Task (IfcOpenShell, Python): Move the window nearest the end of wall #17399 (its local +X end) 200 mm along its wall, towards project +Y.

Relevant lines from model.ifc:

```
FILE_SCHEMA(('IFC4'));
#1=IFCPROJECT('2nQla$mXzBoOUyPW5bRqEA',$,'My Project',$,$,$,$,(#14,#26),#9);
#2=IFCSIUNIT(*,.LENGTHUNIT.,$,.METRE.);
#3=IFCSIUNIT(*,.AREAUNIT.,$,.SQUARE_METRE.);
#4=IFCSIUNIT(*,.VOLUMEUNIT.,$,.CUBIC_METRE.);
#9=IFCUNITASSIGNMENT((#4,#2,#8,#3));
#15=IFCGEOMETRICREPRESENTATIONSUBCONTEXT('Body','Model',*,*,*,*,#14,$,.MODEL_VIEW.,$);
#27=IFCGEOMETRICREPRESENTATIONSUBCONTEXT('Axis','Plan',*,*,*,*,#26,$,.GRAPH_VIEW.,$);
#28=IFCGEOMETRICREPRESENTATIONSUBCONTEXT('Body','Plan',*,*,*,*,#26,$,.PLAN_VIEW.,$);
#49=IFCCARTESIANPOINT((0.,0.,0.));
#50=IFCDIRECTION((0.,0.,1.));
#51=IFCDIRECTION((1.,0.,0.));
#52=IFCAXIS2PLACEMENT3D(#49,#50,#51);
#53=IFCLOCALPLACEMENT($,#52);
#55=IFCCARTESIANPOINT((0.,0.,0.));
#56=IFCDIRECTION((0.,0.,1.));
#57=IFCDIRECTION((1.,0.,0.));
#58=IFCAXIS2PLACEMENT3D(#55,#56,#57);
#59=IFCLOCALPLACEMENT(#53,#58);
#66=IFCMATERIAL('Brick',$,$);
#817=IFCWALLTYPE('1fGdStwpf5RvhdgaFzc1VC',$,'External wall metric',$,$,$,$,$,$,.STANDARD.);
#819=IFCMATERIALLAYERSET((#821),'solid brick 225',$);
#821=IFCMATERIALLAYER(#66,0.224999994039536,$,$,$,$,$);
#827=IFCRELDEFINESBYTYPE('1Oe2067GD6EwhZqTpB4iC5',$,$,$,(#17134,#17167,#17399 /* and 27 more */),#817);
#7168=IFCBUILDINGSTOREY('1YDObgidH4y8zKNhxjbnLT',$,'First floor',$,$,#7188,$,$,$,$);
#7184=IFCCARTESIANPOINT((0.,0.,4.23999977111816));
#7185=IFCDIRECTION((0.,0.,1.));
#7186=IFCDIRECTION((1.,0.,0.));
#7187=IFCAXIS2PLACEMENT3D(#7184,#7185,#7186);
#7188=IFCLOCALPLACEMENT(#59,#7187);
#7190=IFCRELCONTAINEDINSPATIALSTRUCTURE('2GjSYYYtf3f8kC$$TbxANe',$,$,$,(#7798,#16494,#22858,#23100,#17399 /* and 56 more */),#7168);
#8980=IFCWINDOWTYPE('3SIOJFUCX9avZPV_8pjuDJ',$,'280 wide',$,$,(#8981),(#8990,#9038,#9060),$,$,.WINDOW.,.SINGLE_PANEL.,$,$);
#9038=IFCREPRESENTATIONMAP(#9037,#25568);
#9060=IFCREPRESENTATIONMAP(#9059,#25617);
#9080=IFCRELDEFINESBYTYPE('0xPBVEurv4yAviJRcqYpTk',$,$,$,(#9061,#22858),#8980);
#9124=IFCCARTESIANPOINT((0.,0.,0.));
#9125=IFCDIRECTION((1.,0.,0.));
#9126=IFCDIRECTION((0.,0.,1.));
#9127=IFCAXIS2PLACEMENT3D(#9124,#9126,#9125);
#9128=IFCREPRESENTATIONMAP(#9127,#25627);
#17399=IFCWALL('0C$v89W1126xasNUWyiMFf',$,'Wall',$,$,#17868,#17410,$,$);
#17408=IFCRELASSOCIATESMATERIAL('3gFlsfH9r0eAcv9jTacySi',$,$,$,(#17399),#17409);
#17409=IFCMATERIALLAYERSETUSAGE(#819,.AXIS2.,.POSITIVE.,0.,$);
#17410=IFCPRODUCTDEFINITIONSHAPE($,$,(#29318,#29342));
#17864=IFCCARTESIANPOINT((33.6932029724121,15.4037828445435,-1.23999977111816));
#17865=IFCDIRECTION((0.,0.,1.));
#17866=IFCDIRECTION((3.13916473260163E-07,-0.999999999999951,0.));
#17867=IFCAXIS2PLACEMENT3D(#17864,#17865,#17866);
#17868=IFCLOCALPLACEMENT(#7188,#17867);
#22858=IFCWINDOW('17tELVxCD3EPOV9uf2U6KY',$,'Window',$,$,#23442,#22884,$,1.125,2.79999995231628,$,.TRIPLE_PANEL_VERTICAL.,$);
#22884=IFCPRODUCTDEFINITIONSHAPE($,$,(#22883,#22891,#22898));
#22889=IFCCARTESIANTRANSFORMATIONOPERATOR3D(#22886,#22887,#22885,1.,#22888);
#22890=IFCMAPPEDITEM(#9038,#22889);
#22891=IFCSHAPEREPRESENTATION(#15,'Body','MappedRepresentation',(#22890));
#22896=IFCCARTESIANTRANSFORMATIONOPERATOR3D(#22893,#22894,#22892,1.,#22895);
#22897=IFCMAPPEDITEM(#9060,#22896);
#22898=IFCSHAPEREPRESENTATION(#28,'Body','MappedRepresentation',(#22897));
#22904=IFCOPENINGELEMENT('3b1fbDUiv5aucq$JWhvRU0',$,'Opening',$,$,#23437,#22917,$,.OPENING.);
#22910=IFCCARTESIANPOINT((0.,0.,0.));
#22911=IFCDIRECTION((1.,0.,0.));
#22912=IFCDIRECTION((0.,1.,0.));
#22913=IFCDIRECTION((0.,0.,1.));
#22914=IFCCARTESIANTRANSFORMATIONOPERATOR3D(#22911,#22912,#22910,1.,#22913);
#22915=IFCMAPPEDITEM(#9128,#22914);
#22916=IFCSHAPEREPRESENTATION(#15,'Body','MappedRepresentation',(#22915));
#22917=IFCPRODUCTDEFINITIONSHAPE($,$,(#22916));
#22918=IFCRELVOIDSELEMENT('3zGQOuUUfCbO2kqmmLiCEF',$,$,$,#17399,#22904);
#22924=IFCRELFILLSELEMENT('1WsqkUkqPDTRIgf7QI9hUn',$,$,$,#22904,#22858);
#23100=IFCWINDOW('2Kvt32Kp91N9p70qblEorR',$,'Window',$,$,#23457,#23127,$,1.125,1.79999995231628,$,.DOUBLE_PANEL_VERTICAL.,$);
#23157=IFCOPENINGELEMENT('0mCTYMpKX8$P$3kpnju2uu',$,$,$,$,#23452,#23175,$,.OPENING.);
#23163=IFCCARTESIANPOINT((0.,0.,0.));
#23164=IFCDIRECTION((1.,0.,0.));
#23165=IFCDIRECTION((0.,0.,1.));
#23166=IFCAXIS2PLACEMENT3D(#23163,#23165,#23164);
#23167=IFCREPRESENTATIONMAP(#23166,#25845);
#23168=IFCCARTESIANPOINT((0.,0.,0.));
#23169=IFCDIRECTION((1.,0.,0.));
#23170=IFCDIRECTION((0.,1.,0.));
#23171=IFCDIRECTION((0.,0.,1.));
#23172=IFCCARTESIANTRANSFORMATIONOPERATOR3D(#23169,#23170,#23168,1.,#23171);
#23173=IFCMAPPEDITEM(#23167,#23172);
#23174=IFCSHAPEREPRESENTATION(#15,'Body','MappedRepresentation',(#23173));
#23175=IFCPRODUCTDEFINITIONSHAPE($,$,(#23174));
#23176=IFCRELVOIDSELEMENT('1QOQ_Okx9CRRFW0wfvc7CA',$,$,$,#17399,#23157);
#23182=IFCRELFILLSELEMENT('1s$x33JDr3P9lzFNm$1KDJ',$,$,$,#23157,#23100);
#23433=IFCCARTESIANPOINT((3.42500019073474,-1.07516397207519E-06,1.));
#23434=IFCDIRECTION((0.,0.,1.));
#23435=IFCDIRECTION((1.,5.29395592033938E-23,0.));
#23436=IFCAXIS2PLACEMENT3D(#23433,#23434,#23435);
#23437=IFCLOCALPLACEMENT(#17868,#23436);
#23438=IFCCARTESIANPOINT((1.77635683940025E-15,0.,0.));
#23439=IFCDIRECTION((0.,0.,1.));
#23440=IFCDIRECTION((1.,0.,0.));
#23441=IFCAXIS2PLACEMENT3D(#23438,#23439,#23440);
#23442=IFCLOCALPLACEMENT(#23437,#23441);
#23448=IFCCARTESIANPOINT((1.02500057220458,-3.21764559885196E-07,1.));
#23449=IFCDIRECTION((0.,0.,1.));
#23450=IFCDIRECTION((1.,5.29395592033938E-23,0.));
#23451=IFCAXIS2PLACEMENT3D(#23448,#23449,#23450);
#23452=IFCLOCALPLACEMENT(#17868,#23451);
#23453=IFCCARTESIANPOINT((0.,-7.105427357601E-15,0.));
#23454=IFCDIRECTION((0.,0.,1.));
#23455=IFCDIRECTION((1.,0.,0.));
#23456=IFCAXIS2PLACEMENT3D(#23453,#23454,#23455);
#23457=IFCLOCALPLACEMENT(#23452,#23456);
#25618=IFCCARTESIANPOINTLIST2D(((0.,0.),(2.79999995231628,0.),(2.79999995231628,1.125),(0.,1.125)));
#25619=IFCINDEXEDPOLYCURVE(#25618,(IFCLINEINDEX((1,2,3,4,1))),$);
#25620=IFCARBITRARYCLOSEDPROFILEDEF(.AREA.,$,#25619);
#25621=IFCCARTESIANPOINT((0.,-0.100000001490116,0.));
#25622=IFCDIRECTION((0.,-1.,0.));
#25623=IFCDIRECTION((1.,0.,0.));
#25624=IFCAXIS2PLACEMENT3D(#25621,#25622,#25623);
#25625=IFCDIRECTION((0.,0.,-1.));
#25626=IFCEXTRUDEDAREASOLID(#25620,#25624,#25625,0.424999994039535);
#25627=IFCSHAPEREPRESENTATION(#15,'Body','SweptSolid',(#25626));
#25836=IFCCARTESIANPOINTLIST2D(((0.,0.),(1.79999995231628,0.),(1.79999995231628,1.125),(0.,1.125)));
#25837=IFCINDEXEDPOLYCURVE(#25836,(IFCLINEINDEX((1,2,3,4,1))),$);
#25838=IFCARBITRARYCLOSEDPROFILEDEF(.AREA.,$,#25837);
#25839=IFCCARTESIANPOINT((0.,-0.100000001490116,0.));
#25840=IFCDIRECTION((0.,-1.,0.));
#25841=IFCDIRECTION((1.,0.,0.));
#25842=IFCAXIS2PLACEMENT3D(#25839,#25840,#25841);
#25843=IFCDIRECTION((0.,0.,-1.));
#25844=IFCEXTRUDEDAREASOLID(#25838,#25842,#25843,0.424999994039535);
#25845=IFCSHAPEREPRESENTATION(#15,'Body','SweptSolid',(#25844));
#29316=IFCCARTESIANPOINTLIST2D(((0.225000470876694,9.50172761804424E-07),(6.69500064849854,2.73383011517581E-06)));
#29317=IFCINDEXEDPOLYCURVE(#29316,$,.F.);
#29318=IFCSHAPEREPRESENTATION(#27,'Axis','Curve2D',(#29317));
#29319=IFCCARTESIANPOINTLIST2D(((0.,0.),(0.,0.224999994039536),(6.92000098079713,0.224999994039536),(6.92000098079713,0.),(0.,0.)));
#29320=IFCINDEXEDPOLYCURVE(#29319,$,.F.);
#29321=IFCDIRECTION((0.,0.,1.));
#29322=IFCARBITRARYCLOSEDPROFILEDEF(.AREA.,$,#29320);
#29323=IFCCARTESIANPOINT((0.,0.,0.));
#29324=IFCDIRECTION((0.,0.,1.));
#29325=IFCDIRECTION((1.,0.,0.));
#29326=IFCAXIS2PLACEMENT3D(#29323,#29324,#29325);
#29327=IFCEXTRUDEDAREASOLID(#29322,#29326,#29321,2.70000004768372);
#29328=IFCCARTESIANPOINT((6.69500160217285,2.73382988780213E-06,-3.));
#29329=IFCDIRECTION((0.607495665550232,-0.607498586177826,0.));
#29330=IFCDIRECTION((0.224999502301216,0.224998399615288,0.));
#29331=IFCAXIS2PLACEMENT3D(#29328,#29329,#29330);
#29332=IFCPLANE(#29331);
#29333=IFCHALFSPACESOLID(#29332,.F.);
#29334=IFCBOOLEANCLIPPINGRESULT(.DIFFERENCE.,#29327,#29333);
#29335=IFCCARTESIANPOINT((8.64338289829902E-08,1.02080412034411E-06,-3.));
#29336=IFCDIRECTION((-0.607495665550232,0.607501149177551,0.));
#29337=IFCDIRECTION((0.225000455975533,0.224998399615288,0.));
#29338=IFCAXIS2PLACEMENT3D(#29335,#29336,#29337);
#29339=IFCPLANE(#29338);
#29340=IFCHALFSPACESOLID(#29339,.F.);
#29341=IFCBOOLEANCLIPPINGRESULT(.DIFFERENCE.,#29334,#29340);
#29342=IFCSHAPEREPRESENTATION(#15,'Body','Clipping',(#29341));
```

```python
import ifcopenshell
import ifcopenshell.api.geometry
import ifcopenshell.util.placement
import ifcopenshell.util.unit

model = ifcopenshell.open("model.ifc")
unit_scale = ifcopenshell.util.unit.calculate_unit_scale(model)

window = model.by_guid("17tELVxCD3EPOV9uf2U6KY")
opening = window.FillsVoids[0].RelatingOpeningElement
wall = opening.VoidsElements[0].RelatingBuildingElement

wall_matrix = ifcopenshell.util.placement.get_local_placement(wall.ObjectPlacement)
shift = wall_matrix[:3, 0] * -0.2 / unit_scale
before = ifcopenshell.util.placement.get_local_placement(window.ObjectPlacement)[:3, 3].copy()

# The window is placed relative to its opening, so it follows when the opening moves.
matrix = ifcopenshell.util.placement.get_local_placement(opening.ObjectPlacement)
matrix[:3, 3] += shift
ifcopenshell.api.geometry.edit_object_placement(
    model, product=opening, matrix=matrix, is_si=False, should_transform_children=True
)

after = ifcopenshell.util.placement.get_local_placement(window.ObjectPlacement)[:3, 3]
print("window moved by", (after - before).round(3) + 0.0)

model.write("model_rev.ifc")
```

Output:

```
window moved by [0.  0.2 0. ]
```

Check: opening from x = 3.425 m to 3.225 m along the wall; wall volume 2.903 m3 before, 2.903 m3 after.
